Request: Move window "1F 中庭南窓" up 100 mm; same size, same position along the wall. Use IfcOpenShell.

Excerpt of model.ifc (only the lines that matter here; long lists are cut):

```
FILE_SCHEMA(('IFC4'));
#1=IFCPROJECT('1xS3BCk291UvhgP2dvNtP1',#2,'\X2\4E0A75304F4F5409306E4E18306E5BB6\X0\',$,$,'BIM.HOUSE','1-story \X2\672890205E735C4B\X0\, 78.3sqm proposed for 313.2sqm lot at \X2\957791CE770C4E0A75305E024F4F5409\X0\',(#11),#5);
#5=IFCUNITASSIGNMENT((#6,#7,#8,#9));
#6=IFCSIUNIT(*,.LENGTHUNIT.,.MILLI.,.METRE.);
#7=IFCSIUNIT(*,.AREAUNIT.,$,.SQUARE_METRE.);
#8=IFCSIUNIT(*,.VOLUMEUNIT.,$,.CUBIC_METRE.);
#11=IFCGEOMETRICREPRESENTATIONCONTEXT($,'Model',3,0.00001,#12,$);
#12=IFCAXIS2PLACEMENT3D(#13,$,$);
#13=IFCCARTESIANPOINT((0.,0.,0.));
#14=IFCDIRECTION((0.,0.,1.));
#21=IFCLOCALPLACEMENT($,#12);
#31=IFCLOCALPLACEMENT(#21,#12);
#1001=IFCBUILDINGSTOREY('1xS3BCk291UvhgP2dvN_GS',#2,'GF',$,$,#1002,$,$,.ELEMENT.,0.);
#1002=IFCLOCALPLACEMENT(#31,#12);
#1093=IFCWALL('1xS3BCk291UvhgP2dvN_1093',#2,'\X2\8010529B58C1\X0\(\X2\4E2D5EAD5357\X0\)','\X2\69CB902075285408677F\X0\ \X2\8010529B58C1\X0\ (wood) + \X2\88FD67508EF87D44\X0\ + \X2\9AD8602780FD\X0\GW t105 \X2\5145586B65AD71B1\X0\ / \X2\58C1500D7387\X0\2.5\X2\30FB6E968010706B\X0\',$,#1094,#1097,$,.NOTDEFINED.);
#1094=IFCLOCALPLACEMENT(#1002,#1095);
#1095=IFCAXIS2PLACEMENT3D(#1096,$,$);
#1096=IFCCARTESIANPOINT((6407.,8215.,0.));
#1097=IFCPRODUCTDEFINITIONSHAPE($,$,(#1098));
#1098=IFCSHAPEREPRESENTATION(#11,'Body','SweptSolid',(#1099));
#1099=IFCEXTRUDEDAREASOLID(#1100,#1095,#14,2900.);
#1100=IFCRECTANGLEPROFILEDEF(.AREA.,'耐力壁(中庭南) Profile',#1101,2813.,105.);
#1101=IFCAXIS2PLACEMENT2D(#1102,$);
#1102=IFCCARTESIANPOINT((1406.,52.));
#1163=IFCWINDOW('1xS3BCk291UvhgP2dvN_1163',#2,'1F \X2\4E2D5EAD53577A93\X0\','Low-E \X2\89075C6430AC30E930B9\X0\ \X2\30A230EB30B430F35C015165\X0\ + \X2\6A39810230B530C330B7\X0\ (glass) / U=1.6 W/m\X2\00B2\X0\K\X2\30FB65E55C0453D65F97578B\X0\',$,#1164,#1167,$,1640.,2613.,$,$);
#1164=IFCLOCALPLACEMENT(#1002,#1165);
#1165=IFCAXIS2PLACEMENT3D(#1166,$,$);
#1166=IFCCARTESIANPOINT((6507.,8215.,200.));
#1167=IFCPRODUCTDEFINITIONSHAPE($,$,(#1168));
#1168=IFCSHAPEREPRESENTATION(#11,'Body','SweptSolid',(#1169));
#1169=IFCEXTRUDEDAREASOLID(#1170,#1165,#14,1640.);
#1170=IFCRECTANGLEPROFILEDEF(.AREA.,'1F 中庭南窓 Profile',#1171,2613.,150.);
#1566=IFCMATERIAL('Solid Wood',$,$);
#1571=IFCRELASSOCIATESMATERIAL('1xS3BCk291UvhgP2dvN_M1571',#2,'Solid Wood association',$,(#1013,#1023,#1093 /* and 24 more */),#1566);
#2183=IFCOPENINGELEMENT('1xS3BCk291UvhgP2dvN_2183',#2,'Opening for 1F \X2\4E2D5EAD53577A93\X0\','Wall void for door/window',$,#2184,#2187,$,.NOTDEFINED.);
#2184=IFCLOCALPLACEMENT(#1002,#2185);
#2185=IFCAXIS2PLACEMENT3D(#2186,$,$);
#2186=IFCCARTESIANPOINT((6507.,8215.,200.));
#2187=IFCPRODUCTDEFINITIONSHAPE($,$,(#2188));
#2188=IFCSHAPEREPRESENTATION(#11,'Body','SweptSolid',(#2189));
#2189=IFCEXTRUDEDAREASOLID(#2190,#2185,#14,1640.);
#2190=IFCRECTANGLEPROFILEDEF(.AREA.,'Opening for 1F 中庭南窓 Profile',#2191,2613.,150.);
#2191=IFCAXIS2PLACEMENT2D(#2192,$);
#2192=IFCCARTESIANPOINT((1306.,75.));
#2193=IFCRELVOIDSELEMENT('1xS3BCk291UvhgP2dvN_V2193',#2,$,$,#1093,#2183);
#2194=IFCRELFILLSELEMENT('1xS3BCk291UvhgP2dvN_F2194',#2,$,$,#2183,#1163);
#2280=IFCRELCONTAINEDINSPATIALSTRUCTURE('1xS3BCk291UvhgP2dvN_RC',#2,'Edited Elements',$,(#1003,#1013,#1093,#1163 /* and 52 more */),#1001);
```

```python
import numpy as np
import ifcopenshell
import ifcopenshell.api.geometry
import ifcopenshell.util.placement
import ifcopenshell.util.unit

model = ifcopenshell.open("model.ifc")
unit_scale = ifcopenshell.util.unit.calculate_unit_scale(model)

window = model.by_id(1163)
opening = window.FillsVoids[0].RelatingOpeningElement
dz = 0.1 / unit_scale

shift = np.array([0.0, 0.0, dz])
# The window is not placed relative to its opening, so move both.
for product in (opening, window):
    matrix = ifcopenshell.util.placement.get_local_placement(product.ObjectPlacement)
    matrix[:3, 3] += shift
    ifcopenshell.api.geometry.edit_object_placement(model, product=product, matrix=matrix, is_si=False)

print(f"moved by {dz * unit_scale:+.3f} m")

model.write("model-out.ifc")
```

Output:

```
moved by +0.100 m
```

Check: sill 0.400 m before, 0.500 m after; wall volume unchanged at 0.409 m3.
